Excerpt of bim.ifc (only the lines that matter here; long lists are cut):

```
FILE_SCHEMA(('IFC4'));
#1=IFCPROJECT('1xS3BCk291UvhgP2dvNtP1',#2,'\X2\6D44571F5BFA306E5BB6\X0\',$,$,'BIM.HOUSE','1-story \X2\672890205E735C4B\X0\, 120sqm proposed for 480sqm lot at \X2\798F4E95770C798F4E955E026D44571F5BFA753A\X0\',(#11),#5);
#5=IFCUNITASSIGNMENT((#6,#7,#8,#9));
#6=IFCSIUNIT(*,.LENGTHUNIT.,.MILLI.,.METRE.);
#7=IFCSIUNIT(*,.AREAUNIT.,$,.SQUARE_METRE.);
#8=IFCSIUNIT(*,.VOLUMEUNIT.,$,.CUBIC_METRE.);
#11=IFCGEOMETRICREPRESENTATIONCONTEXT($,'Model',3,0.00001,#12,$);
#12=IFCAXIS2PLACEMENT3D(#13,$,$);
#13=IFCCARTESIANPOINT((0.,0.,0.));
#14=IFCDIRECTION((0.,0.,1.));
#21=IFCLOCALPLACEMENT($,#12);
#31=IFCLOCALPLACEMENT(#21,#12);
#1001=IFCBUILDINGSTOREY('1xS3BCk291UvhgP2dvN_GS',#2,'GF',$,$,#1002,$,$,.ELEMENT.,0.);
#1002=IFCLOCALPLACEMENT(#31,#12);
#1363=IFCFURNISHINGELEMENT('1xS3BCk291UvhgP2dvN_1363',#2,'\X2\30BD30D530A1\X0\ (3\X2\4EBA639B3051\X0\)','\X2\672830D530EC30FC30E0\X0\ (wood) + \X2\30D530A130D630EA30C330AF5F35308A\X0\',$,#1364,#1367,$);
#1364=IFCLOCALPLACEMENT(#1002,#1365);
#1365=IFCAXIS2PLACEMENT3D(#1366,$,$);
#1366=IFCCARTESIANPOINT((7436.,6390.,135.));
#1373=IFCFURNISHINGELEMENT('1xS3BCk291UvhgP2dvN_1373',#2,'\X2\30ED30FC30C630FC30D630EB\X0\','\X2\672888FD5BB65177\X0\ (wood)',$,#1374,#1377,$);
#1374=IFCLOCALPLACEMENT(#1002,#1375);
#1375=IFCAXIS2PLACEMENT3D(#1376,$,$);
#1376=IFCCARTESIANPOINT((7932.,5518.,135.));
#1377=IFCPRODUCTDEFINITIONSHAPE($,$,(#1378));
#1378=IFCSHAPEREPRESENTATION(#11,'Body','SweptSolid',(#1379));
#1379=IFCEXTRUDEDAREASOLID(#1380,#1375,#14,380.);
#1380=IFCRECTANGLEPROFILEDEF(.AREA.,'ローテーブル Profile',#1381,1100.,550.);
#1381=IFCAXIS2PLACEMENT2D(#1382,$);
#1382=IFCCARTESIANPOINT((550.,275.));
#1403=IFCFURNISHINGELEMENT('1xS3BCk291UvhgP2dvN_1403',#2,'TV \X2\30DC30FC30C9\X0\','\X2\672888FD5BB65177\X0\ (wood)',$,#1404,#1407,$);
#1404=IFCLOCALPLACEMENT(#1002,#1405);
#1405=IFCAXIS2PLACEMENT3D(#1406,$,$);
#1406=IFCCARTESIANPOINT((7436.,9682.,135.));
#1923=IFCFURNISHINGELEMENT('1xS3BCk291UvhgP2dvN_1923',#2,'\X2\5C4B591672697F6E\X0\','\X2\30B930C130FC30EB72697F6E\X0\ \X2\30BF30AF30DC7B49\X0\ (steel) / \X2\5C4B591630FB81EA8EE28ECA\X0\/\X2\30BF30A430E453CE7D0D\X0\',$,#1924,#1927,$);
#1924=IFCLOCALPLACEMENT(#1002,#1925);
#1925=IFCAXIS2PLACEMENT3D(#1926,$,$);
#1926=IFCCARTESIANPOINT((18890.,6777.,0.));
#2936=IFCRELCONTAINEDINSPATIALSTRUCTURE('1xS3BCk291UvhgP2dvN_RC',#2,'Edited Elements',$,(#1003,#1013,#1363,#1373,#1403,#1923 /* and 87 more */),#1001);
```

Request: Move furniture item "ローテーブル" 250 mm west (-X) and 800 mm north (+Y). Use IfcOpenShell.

```python
import ifcopenshell
import ifcopenshell.api.geometry
import ifcopenshell.util.placement

model = ifcopenshell.open("bim.ifc")

item = model.by_guid("1xS3BCk291UvhgP2dvN_1373")
matrix = ifcopenshell.util.placement.get_local_placement(item.ObjectPlacement)
matrix[0, 3] -= 250.0
matrix[1, 3] += 800.0
ifcopenshell.api.geometry.edit_object_placement(model, product=item, matrix=matrix, is_si=False)

print(ifcopenshell.util.placement.get_local_placement(item.ObjectPlacement).round(3) + 0.0)

model.write("bim_updated.ifc")
```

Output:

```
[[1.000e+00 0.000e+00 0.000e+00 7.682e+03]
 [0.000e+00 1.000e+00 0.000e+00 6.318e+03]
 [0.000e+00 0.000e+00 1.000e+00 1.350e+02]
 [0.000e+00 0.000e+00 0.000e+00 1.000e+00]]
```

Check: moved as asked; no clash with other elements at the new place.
